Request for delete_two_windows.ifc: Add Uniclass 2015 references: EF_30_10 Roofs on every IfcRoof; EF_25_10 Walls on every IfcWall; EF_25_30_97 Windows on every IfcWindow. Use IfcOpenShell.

First a look at what the model holds.

```python
import ifcopenshell

model = ifcopenshell.open("delete_two_windows.ifc")
print(model.schema)
print("classifications:", [c.Name for c in model.by_type("IfcClassification")])
for ifc_class in ("IfcDoor", "IfcRoof", "IfcStair", "IfcWall", "IfcWindow"):
    print(ifc_class, len(model.by_type(ifc_class)))
```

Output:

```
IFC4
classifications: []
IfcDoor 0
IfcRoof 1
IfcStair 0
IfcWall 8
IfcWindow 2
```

```python
import ifcopenshell
import ifcopenshell.api.classification

model = ifcopenshell.open("delete_two_windows.ifc")

system = ifcopenshell.api.classification.add_classification(model, classification="Uniclass 2015")

codes = {
    "IfcRoof": ("EF_30_10", "Roofs"),
    "IfcWall": ("EF_25_10", "Walls"),
    "IfcWindow": ("EF_25_30_97", "Windows"),
}
for ifc_class, (code, name) in codes.items():
    products = model.by_type(ifc_class)
    ifcopenshell.api.classification.add_reference(
        model, products=products, classification=system, identification=code, name=name
    )
    print(code, len(products))

model.write("delete_two_windows_rev.ifc")
```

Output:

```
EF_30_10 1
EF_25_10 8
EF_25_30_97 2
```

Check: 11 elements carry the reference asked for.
